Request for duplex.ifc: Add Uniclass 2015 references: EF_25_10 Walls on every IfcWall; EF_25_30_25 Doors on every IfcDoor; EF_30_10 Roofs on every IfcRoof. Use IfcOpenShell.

First a look at what the model holds.

```python
import ifcopenshell

model = ifcopenshell.open("duplex.ifc")
print(model.schema)
print("classifications:", [c.Name for c in model.by_type("IfcClassification")])
for ifc_class in ("IfcDoor", "IfcRoof", "IfcStair", "IfcWall", "IfcWindow"):
    print(ifc_class, len(model.by_type(ifc_class)))
```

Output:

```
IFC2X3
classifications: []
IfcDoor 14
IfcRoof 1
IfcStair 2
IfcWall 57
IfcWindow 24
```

```python
import ifcopenshell
import ifcopenshell.api.classification

model = ifcopenshell.open("duplex.ifc")

# IFC2X3 requires Source and Edition and has no link from the project to the system.
system = model.create_entity("IfcClassification", Source="NBS", Edition="2015", Name="Uniclass 2015")

codes = {
    "IfcWall": ("EF_25_10", "Walls"),
    "IfcDoor": ("EF_25_30_25", "Doors"),
    "IfcRoof": ("EF_30_10", "Roofs"),
}
for ifc_class, (code, name) in codes.items():
    products = model.by_type(ifc_class)
    ifcopenshell.api.classification.add_reference(
        model, products=products, classification=system, identification=code, name=name
    )
    print(code, len(products))

model.write("duplex-out.ifc")
```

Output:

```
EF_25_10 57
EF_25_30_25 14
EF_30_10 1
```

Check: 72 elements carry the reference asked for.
